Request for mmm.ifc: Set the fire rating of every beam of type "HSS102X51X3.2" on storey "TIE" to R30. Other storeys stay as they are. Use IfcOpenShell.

First a look at what the model holds.

```python
import ifcopenshell
import ifcopenshell.util.element

model = ifcopenshell.open("mmm.ifc")
print(model.schema)
storey = next(s for s in model.by_type("IfcBuildingStorey") if s.Name == "TIE")
beams = [e for e in ifcopenshell.util.element.get_decomposition(storey) if e.is_a("IfcBeam")]
seen = {}
for e in beams:
    element_type = ifcopenshell.util.element.get_type(e)
    key = (element_type.Name if element_type != e and element_type else None, ifcopenshell.util.element.get_pset(e, "Pset_BeamCommon", "FireRating"))
    seen[key] = seen.get(key, 0) + 1
for (name, value), count in sorted(seen.items(), key=str):
    print(count, "x", name, "|", value)
```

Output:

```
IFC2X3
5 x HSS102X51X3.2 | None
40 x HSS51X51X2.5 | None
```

```python
import ifcopenshell
import ifcopenshell.api.pset
import ifcopenshell.util.element

model = ifcopenshell.open("mmm.ifc")

storey = next(s for s in model.by_type("IfcBuildingStorey") if s.Name == "TIE")
beams = [e for e in ifcopenshell.util.element.get_decomposition(storey) if e.is_a("IfcBeam")]

count = 0
for e in beams:
    element_type = ifcopenshell.util.element.get_type(e)
    if element_type in (None, e) or element_type.Name != "HSS102X51X3.2":
        continue
    found = ifcopenshell.util.element.get_pset(e, "Pset_BeamCommon", should_inherit=False)
    if found:
        pset = model.by_id(found["id"])
        if len(ifcopenshell.util.element.get_elements_by_pset(pset)) > 1:
            pset = ifcopenshell.api.pset.unshare_pset(model, products=[e], pset=pset)[0]
    else:
        pset = ifcopenshell.api.pset.add_pset(model, product=e, name="Pset_BeamCommon")
    ifcopenshell.api.pset.edit_pset(model, pset=pset, properties={"FireRating": "R30"})
    count += 1

print(count, "beams updated")

model.write("mmm_rev.ifc")
```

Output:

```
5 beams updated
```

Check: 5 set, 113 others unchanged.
